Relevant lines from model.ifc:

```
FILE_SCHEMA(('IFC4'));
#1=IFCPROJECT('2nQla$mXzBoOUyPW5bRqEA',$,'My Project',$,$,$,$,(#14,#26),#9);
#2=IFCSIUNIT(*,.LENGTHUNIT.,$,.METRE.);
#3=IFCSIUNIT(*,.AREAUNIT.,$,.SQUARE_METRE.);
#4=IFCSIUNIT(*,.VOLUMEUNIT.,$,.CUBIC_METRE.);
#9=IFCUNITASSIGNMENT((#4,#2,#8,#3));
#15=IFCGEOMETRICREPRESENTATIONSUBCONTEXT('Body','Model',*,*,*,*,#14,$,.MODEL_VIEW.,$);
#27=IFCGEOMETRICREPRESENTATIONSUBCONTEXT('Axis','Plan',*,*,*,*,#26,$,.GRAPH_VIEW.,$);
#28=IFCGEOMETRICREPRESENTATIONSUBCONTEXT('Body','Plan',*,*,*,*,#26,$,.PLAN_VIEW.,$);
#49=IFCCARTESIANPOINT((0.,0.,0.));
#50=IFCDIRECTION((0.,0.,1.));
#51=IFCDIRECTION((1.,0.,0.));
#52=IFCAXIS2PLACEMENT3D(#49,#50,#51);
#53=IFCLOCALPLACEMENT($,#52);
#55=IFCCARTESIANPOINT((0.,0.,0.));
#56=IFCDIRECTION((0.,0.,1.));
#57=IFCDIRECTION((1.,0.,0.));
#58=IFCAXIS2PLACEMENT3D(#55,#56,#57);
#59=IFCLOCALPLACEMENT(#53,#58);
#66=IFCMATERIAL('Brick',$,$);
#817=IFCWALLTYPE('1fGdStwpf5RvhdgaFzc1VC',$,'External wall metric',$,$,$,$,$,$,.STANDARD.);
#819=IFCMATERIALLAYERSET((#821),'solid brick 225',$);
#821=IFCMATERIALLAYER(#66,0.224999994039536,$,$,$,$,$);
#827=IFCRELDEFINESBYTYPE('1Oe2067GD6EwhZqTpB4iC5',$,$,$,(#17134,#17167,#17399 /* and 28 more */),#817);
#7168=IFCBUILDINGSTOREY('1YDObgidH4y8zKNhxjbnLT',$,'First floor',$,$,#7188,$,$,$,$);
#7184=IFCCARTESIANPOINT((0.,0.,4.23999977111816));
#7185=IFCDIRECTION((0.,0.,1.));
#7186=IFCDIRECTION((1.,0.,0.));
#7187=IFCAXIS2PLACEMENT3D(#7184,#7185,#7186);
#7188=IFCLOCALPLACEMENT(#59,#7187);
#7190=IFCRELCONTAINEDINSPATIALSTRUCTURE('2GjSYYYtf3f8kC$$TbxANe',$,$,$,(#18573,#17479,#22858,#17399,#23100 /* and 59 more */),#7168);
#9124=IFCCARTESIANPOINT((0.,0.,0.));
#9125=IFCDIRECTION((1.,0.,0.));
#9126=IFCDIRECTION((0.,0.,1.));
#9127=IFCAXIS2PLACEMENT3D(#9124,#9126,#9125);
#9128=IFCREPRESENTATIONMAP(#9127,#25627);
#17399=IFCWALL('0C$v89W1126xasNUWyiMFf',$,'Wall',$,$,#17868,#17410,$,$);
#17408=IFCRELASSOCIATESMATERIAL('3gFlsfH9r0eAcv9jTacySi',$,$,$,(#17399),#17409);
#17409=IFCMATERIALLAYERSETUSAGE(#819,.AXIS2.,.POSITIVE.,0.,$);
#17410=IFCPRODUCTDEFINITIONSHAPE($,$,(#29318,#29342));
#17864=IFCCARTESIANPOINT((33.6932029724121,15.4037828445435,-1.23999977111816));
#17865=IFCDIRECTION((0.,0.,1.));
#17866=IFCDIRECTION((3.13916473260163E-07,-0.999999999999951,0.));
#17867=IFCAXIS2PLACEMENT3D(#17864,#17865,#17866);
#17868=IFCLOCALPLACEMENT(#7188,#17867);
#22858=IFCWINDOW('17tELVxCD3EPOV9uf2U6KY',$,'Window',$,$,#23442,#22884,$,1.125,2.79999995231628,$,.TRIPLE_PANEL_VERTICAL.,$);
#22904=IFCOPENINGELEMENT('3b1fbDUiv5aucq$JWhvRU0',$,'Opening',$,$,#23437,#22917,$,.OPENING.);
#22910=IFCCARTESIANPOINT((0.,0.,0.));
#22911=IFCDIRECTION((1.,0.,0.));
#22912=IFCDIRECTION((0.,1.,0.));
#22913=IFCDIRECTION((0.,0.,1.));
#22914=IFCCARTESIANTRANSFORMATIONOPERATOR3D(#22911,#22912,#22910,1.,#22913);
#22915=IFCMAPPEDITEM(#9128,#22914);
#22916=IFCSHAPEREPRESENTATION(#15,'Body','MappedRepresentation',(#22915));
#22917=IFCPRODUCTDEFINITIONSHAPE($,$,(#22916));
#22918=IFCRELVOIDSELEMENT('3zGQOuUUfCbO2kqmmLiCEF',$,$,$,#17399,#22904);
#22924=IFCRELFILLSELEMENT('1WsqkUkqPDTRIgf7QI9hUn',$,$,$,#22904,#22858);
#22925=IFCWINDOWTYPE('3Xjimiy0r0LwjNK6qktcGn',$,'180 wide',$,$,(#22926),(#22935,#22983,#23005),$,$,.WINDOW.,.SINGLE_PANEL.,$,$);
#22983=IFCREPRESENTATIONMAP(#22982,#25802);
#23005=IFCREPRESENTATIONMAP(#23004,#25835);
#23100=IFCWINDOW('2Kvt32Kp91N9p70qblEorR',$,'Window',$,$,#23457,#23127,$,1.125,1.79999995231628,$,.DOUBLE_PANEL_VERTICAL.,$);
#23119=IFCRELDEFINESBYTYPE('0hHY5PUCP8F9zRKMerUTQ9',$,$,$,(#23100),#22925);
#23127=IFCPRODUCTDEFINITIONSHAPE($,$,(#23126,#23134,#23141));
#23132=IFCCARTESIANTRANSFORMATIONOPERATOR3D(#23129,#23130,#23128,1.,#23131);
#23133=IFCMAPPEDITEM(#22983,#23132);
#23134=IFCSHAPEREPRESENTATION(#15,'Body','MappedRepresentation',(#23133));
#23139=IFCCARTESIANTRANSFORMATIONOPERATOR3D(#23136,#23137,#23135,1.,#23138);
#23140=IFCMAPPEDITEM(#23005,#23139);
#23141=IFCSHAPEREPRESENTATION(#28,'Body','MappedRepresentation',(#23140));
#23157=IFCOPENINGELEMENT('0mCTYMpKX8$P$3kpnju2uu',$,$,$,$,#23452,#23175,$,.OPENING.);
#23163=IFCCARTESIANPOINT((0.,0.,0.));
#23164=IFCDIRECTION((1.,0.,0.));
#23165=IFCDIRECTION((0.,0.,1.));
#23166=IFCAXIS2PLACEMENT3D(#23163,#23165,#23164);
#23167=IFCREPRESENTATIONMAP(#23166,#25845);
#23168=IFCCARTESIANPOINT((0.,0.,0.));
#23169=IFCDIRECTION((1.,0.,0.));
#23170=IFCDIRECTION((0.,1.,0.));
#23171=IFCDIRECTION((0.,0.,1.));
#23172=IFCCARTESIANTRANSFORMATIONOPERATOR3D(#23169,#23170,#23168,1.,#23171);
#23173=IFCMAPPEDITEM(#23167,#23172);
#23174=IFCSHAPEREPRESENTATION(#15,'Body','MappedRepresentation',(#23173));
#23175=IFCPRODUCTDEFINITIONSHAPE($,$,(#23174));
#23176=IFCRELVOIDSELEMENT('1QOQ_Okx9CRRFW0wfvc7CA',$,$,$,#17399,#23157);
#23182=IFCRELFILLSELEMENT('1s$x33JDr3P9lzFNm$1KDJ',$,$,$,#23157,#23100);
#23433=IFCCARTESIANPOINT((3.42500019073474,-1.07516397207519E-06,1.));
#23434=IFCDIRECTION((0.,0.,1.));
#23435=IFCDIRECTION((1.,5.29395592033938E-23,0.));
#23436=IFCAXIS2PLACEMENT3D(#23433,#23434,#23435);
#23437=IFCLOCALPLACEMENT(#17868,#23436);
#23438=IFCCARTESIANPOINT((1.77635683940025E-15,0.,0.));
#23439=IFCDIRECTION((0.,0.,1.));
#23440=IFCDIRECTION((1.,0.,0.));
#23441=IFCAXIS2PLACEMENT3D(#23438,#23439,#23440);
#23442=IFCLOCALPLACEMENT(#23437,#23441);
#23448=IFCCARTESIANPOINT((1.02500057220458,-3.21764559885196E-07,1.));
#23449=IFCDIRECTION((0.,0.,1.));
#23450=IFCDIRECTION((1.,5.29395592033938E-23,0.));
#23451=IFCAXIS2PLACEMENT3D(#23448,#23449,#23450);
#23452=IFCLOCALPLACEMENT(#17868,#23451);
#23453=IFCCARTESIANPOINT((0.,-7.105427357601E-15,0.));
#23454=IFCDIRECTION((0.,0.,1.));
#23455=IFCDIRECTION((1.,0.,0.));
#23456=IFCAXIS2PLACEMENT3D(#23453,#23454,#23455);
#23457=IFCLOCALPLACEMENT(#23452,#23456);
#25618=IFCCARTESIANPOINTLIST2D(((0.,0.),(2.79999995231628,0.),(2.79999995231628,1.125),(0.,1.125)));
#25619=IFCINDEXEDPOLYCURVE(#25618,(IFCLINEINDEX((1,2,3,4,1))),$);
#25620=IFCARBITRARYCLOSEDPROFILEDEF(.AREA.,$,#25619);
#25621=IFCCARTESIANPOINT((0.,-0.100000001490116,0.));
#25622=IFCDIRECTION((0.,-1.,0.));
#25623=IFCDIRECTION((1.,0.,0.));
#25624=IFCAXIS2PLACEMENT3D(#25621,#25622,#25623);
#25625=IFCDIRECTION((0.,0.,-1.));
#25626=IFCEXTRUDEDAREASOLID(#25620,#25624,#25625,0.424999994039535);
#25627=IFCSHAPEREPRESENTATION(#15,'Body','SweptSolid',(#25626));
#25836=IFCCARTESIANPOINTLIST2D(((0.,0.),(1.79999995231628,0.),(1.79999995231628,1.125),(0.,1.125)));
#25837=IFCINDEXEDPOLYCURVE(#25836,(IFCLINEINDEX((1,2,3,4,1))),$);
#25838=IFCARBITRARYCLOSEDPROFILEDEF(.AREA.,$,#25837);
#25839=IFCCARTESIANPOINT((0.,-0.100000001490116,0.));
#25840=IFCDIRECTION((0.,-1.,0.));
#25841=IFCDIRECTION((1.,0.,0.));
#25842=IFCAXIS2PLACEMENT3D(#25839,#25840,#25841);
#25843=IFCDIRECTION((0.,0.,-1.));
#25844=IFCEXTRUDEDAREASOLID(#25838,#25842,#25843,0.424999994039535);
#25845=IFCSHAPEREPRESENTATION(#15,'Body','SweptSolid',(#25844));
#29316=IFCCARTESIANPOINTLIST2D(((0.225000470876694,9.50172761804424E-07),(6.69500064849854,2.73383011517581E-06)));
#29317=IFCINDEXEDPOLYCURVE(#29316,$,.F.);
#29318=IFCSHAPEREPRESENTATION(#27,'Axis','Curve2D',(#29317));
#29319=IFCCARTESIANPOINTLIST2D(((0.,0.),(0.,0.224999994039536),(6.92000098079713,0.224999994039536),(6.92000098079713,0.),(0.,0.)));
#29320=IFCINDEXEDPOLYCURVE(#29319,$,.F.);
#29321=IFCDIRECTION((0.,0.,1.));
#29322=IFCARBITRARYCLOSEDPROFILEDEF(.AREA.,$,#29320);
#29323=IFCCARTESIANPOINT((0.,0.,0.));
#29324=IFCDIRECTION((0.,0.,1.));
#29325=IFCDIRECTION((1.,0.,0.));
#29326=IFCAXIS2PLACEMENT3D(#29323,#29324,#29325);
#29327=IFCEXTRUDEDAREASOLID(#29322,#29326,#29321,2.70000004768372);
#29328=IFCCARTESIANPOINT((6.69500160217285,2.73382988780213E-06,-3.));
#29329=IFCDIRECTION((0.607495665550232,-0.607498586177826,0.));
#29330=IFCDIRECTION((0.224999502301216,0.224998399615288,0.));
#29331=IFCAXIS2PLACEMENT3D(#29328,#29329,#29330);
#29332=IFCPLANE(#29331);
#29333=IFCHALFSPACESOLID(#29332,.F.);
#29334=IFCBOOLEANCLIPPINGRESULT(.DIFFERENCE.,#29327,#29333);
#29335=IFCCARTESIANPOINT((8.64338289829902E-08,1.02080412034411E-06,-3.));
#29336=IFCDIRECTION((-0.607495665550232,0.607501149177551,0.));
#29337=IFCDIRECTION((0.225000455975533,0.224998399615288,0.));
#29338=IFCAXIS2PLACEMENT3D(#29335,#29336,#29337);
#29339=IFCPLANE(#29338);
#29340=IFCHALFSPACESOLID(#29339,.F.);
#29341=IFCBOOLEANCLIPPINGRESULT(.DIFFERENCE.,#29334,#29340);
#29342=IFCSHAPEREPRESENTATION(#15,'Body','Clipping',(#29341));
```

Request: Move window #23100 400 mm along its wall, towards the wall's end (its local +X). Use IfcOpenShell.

```python
import ifcopenshell
import ifcopenshell.api.geometry
import ifcopenshell.util.placement
import ifcopenshell.util.unit

model = ifcopenshell.open("model.ifc")
unit_scale = ifcopenshell.util.unit.calculate_unit_scale(model)

window = model.by_id(23100)
opening = window.FillsVoids[0].RelatingOpeningElement
wall = opening.VoidsElements[0].RelatingBuildingElement

wall_matrix = ifcopenshell.util.placement.get_local_placement(wall.ObjectPlacement)
shift = wall_matrix[:3, 0] * 0.4 / unit_scale
before = ifcopenshell.util.placement.get_local_placement(window.ObjectPlacement)[:3, 3].copy()

# The window is placed relative to its opening, so it follows when the opening moves.
matrix = ifcopenshell.util.placement.get_local_placement(opening.ObjectPlacement)
matrix[:3, 3] += shift
ifcopenshell.api.geometry.edit_object_placement(
    model, product=opening, matrix=matrix, is_si=False, should_transform_children=True
)

after = ifcopenshell.util.placement.get_local_placement(window.ObjectPlacement)[:3, 3]
print("window moved by", (after - before).round(3) + 0.0)

model.write("model_rev.ifc")
```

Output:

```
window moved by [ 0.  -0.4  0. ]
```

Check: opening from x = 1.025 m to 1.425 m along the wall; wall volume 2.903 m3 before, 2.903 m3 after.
